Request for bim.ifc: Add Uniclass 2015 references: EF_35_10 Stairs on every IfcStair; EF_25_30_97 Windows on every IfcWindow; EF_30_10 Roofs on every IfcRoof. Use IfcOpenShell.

First a look at what the model holds.

```python
import ifcopenshell

model = ifcopenshell.open("bim.ifc")
print(model.schema)
print("classifications:", [c.Name for c in model.by_type("IfcClassification")])
for ifc_class in ("IfcDoor", "IfcRoof", "IfcStair", "IfcWall", "IfcWindow"):
    print(ifc_class, len(model.by_type(ifc_class)))
```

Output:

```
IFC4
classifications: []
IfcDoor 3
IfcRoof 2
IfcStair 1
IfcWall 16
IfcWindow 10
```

```python
import ifcopenshell
import ifcopenshell.api.classification

model = ifcopenshell.open("bim.ifc")

system = ifcopenshell.api.classification.add_classification(model, classification="Uniclass 2015")

codes = {
    "IfcStair": ("EF_35_10", "Stairs"),
    "IfcWindow": ("EF_25_30_97", "Windows"),
    "IfcRoof": ("EF_30_10", "Roofs"),
}
for ifc_class, (code, name) in codes.items():
    products = model.by_type(ifc_class)
    ifcopenshell.api.classification.add_reference(
        model, products=products, classification=system, identification=code, name=name
    )
    print(code, len(products))

model.write("bim_edited.ifc")
```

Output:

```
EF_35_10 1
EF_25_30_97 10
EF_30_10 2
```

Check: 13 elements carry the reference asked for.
